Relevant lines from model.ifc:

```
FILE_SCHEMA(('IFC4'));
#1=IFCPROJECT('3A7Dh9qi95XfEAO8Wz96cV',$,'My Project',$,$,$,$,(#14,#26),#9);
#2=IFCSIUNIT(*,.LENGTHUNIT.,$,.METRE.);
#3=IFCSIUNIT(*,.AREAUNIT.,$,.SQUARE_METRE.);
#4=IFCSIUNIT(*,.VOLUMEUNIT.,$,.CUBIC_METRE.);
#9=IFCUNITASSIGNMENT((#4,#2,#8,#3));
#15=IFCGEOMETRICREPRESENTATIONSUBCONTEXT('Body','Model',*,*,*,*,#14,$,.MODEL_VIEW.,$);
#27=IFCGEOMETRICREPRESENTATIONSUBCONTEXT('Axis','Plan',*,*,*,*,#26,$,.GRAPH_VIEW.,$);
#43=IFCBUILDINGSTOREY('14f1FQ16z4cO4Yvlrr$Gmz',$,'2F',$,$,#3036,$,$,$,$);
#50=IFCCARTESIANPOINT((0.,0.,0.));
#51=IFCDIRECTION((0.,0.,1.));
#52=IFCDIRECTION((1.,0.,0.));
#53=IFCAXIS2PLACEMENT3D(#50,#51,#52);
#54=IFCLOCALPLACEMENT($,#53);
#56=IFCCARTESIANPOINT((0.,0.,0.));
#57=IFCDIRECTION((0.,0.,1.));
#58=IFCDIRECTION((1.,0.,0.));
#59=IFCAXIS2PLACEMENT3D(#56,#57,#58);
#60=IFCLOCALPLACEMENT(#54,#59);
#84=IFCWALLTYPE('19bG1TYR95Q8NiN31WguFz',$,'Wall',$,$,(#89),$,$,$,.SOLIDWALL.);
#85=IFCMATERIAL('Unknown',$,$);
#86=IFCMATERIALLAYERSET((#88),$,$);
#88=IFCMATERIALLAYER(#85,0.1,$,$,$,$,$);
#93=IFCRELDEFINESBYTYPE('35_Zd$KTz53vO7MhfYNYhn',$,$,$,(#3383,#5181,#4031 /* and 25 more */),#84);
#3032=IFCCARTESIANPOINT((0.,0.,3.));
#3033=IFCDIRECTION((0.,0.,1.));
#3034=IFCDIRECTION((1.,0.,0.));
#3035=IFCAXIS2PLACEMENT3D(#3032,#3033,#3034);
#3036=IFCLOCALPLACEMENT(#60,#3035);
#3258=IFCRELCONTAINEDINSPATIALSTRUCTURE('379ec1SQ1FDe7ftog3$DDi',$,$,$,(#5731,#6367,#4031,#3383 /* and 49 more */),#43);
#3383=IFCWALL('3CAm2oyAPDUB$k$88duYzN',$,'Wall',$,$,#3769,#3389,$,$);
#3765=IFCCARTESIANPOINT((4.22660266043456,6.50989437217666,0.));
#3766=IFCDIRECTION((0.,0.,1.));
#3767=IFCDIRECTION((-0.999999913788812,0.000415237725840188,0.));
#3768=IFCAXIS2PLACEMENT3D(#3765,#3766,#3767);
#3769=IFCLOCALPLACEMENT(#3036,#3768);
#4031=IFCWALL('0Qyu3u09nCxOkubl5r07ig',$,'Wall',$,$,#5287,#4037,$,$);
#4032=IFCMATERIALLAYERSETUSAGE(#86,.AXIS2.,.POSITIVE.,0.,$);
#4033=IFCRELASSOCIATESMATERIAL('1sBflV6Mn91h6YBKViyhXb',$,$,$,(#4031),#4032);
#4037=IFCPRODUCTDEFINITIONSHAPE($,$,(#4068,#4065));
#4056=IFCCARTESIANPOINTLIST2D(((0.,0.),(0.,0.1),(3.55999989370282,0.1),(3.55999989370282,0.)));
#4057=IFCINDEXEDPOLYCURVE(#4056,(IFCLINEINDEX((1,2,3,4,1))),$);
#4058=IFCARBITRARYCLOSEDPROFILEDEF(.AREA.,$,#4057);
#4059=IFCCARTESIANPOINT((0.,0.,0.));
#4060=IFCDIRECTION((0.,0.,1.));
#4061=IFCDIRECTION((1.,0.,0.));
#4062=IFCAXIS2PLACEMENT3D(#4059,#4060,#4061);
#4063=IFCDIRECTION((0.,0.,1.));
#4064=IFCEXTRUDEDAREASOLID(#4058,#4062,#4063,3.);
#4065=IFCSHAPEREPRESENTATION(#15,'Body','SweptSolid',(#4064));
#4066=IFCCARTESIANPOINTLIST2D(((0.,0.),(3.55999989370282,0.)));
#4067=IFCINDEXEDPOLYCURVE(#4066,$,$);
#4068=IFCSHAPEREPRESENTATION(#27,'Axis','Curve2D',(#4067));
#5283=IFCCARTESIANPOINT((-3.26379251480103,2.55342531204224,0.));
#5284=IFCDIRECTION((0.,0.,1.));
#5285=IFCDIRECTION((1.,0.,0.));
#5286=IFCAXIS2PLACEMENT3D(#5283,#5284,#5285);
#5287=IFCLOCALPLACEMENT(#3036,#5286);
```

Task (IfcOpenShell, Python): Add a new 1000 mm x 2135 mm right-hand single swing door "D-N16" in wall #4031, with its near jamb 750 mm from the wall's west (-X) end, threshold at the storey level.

```python
import numpy as np
import ifcopenshell
import ifcopenshell.api.feature
import ifcopenshell.api.geometry
import ifcopenshell.api.root
import ifcopenshell.api.spatial
import ifcopenshell.geom
import ifcopenshell.util.element
import ifcopenshell.util.placement
import ifcopenshell.util.representation
import ifcopenshell.util.shape
import ifcopenshell.util.unit

model = ifcopenshell.open("model.ifc")
unit_scale = ifcopenshell.util.unit.calculate_unit_scale(model)
settings = ifcopenshell.geom.settings()


def volume(element):
    """Net volume in cubic metres, openings subtracted."""
    shape = ifcopenshell.geom.create_shape(settings, element)
    return ifcopenshell.util.shape.get_volume(shape.geometry)


wall = model.by_id(4031)
storey = ifcopenshell.util.element.get_container(wall, ifc_class="IfcBuildingStorey")
context = ifcopenshell.util.representation.get_context(model, "Model", "Body", "MODEL_VIEW")
before = volume(wall)

width, height, from_end, sill = 1, 2.135, 0.75, 0.0  # metres

# The wall runs along its own X axis, and the end named is its -X end.
wall_shape = ifcopenshell.geom.create_shape(settings, wall)
x, y, z = ifcopenshell.util.shape.get_vertices(wall_shape.geometry).T
start = x.min() + from_end
face, thickness = float(y.min()), float(y.max() - y.min())
wall_matrix = ifcopenshell.util.placement.get_local_placement(wall.ObjectPlacement)
level = ifcopenshell.util.placement.get_local_placement(storey.ObjectPlacement)[2, 3]


def in_wall(x, y):
    """Placement at x, y metres in the wall's axes, at sill height."""
    matrix = wall_matrix.copy()
    matrix[:, 3] = wall_matrix @ np.array([x / unit_scale, y / unit_scale, 0.0, 1.0])
    matrix[2, 3] = level + sill / unit_scale
    return matrix


# Opening: a box that overshoots both wall faces by 50 mm.
opening = ifcopenshell.api.root.create_entity(model, ifc_class="IfcOpeningElement", predefined_type="OPENING")
box = ifcopenshell.api.geometry.add_wall_representation(
    model, context=context, length=width, height=height, thickness=thickness + 0.1
)
ifcopenshell.api.geometry.assign_representation(model, product=opening, representation=box)
ifcopenshell.api.geometry.edit_object_placement(model, product=opening, matrix=in_wall(start, face - 0.05), is_si=False)
ifcopenshell.api.feature.add_feature(model, feature=opening, element=wall)

door = ifcopenshell.api.root.create_entity(model, ifc_class="IfcDoor", name="D-N16", predefined_type="DOOR")
door.OverallWidth, door.OverallHeight = width / unit_scale, height / unit_scale
door.OperationType = "SINGLE_SWING_RIGHT"
body = ifcopenshell.api.geometry.add_door_representation(
    model,
    context=context,
    overall_width=door.OverallWidth,
    overall_height=door.OverallHeight,
    operation_type="SINGLE_SWING_RIGHT",
    lining_properties={"LiningDepth": thickness / unit_scale, "ThresholdDepth": thickness / unit_scale},
)
ifcopenshell.api.geometry.assign_representation(model, product=door, representation=body)
ifcopenshell.api.spatial.assign_container(model, products=[door], relating_structure=storey)
ifcopenshell.api.feature.add_filling(model, opening=opening, element=door)

# The lining spans the wall, so the door starts at the wall face.
ifcopenshell.api.geometry.edit_object_placement(model, product=door, matrix=in_wall(start, face), is_si=False)

after = volume(wall)

print(f"wall volume {before:.3f} -> {after:.3f} m3")

model.write("model-out.ifc")
```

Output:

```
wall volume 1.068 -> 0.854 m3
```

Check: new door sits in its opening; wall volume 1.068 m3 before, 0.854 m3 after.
